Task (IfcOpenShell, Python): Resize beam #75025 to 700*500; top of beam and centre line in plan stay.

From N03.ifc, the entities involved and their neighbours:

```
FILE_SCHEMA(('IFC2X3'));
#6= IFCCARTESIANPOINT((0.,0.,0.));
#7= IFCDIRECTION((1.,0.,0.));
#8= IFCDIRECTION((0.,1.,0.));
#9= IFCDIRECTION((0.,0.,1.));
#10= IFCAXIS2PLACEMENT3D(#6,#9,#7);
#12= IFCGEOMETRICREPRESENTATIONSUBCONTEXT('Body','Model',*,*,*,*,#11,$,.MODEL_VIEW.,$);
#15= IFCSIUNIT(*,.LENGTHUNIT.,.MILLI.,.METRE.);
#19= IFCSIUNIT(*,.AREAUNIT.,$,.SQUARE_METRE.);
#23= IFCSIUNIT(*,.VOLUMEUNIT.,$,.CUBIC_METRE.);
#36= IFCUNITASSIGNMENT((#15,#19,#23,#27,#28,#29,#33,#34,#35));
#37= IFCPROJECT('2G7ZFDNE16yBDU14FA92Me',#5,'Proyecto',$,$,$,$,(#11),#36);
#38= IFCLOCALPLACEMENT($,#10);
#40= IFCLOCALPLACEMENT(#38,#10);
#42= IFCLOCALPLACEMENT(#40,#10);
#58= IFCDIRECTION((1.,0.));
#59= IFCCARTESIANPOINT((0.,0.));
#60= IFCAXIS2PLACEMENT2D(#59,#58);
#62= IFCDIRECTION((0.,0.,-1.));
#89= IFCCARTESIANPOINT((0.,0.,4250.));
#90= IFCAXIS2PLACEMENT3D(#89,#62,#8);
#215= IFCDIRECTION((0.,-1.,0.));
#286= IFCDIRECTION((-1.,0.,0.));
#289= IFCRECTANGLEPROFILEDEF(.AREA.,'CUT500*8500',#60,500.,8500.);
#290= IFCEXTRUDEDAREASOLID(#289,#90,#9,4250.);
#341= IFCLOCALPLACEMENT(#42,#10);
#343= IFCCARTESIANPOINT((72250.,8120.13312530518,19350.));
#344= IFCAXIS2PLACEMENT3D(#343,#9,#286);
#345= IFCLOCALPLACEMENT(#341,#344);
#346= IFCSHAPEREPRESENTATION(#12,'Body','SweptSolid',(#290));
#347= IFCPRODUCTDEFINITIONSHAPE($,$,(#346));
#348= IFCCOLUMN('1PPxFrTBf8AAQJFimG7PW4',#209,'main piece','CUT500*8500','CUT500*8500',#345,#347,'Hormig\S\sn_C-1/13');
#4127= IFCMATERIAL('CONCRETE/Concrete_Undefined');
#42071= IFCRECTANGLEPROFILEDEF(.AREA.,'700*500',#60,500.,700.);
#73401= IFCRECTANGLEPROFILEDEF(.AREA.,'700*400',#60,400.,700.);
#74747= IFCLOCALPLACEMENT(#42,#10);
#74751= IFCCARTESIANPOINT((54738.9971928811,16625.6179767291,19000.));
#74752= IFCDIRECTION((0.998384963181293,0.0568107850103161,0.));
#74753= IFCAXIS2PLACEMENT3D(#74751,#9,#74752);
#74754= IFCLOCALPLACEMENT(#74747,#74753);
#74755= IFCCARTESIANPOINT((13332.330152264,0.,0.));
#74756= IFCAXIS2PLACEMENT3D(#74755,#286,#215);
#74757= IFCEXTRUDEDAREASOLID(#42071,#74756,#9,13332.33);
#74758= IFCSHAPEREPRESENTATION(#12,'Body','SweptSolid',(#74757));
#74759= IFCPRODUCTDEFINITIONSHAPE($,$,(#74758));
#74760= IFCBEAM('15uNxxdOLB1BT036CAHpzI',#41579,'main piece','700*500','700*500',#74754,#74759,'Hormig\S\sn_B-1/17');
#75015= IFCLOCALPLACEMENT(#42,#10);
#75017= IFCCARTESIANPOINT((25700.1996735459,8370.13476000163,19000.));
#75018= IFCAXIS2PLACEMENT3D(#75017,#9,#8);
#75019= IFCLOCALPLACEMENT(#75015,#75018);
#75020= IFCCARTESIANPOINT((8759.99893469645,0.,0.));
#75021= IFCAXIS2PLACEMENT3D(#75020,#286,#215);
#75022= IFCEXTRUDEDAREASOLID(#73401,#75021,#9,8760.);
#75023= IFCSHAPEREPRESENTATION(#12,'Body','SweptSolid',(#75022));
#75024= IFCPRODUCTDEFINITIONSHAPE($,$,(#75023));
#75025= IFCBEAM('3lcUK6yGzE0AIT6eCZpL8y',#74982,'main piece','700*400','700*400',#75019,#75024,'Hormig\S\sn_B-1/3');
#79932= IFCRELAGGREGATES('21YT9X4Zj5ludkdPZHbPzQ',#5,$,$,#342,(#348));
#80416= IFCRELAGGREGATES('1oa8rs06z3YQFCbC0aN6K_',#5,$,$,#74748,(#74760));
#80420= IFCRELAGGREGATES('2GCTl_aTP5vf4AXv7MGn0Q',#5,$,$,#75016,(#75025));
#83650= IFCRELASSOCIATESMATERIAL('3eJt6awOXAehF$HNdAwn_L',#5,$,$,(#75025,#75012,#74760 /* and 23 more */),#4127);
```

```python
import ifcopenshell
import ifcopenshell.util.element
import ifcopenshell.util.representation

model = ifcopenshell.open("N03.ifc")

member = model.by_guid("3lcUK6yGzE0AIT6eCZpL8y")
source = next(p for p in model.by_type("IfcRectangleProfileDef") if p.ProfileName == "700*500")

body = ifcopenshell.util.representation.get_representation(member, "Model", "Body")
solid = body.Items[0]
old_profile = solid.SweptArea

# Copy the section's sizes but keep this member's own profile position.
profile = ifcopenshell.util.element.copy(model, source)
# Profiles are centred, so shift by half the change in depth to hold the top.
shift = (old_profile.YDim - profile.YDim) / 2
x, y = old_profile.Position.Location.Coordinates
up = (0.0, 1.0)  # upwards, in the solid's own plane
location = model.createIfcCartesianPoint((x + up[0] * shift, y + up[1] * shift))
profile.Position = model.createIfcAxis2Placement2D(location, old_profile.Position.RefDirection)
solid.SweptArea = profile
if not model.get_total_inverses(old_profile):
    ifcopenshell.util.element.remove_deep2(model, old_profile)
member.Description = member.Description.replace("700*400", "700*500")
member.ObjectType = member.ObjectType.replace("700*400", "700*500")

print(solid.SweptArea)

model.write("N03_updated.ifc")
```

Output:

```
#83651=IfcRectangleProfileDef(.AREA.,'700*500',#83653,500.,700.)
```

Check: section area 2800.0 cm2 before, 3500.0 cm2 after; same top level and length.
